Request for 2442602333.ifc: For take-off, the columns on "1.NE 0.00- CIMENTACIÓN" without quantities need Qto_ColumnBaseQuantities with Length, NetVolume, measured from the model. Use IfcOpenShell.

First a look at what the model holds.

```python
import ifcopenshell
import ifcopenshell.util.element
import ifcopenshell.util.unit

model = ifcopenshell.open("2442602333.ifc")
print(model.schema)
for unit_type in ("LENGTHUNIT", "AREAUNIT", "VOLUMEUNIT"):
    print(unit_type, ifcopenshell.util.unit.calculate_unit_scale(model, unit_type))
storey = next(s for s in model.by_type("IfcBuildingStorey") if s.Name == "1.NE 0.00- CIMENTACIÓN")
columns = [e for e in ifcopenshell.util.element.get_decomposition(storey) if e.is_a("IfcColumn")]
for e in sorted(columns, key=lambda e: e.id()):
    print(e.id(), e.is_a(), e.Name, list(ifcopenshell.util.element.get_psets(e, qtos_only=True)), sep=" | ")
```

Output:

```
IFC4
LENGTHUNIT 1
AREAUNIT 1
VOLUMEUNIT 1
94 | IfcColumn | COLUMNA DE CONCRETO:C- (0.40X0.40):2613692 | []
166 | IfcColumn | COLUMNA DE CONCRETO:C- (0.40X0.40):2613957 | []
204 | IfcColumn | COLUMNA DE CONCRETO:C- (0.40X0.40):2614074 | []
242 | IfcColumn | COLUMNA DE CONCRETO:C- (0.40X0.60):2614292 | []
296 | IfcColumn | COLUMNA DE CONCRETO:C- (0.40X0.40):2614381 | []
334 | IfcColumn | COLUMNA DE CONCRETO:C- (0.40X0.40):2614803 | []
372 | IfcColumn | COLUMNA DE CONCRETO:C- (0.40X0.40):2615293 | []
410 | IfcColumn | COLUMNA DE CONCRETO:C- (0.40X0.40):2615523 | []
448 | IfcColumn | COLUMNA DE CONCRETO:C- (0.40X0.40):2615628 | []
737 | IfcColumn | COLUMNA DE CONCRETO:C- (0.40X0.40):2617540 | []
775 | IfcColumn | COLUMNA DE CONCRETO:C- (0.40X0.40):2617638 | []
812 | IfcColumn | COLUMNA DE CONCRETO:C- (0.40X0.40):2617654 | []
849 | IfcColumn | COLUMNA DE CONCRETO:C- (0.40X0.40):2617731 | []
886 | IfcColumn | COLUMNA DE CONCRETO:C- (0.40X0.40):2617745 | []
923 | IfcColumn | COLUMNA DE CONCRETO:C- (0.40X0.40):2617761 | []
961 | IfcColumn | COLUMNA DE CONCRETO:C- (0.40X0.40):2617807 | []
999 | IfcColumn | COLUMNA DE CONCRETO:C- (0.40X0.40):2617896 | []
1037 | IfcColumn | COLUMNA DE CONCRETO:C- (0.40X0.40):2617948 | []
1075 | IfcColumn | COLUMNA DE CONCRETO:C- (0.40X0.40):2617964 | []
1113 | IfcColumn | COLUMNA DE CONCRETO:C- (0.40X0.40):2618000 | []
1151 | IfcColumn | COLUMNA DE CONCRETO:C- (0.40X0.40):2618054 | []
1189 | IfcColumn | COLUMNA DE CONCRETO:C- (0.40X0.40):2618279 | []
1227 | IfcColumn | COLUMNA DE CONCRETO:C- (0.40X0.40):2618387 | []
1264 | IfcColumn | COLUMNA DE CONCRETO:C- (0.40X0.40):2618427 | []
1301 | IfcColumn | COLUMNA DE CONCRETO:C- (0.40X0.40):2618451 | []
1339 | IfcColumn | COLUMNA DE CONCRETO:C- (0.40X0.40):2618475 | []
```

```python
import ifcopenshell
import ifcopenshell.api.pset
import ifcopenshell.geom
import ifcopenshell.util.element
import ifcopenshell.util.shape
import ifcopenshell.util.unit

model = ifcopenshell.open("2442602333.ifc")
unit_scale = ifcopenshell.util.unit.calculate_unit_scale(model)
volume_scale = ifcopenshell.util.unit.calculate_unit_scale(model, "VOLUMEUNIT")
settings = ifcopenshell.geom.settings()

storey = next(s for s in model.by_type("IfcBuildingStorey") if s.Name == "1.NE 0.00- CIMENTACIÓN")
columns = [e for e in ifcopenshell.util.element.get_decomposition(storey) if e.is_a("IfcColumn")]

for e in sorted(columns, key=lambda e: e.id()):
    if ifcopenshell.util.element.get_psets(e, qtos_only=True, should_inherit=False):
        continue
    # Geometry comes back in metres, in the element's own axes.
    shape = ifcopenshell.geom.create_shape(settings, e)
    values = {
        "Length": ifcopenshell.util.shape.get_z(shape.geometry) / unit_scale,
        "NetVolume": ifcopenshell.util.shape.get_volume(shape.geometry) / volume_scale,
    }
    qto = ifcopenshell.api.pset.add_qto(model, product=e, name="Qto_ColumnBaseQuantities")
    ifcopenshell.api.pset.edit_qto(model, qto=qto, properties=values)
    print(e.id(), {k: round(v, 3) for k, v in values.items()})

model.write("2442602333_rev.ifc")
```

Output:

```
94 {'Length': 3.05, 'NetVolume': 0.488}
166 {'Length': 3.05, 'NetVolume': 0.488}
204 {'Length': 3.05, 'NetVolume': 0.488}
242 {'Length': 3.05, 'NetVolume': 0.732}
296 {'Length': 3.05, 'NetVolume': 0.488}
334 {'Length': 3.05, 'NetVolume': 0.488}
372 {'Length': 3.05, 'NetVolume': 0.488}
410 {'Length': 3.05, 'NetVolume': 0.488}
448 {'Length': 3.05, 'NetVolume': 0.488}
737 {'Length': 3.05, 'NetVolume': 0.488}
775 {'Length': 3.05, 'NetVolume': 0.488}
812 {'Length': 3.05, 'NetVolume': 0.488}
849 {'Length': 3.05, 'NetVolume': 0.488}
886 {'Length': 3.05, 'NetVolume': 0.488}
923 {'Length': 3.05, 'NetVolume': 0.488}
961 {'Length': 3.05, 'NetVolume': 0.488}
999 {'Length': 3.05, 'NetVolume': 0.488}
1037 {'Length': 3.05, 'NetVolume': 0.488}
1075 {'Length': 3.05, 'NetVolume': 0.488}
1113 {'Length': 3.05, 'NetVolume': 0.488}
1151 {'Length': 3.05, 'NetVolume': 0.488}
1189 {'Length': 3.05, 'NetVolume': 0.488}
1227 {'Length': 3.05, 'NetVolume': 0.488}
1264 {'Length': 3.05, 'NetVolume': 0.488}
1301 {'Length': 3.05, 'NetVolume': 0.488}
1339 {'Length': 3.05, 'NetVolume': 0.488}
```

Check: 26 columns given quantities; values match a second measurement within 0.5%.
